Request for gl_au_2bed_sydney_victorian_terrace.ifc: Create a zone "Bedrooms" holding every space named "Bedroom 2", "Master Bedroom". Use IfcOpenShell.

First a look at what the model holds.

```python
import ifcopenshell

model = ifcopenshell.open("gl_au_2bed_sydney_victorian_terrace.ifc")
print(model.schema)
seen = {}
for space in model.by_type("IfcSpace"):
    seen[space.LongName] = seen.get(space.LongName, 0) + 1
for name, count in sorted(seen.items(), key=str):
    print(count, "x", name)
print("zones:", [z.Name for z in model.by_type("IfcZone")][:20])
```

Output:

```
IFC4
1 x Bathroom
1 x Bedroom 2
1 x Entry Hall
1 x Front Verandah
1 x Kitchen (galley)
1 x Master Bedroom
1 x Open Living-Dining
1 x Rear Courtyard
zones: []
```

```python
import ifcopenshell
import ifcopenshell.api.group
import ifcopenshell.api.root

model = ifcopenshell.open("gl_au_2bed_sydney_victorian_terrace.ifc")

names = {"Bedroom 2", "Master Bedroom"}
spaces = [s for s in model.by_type("IfcSpace") if s.LongName in names]

zone = ifcopenshell.api.root.create_entity(model, ifc_class="IfcZone", name="Bedrooms")
ifcopenshell.api.group.assign_group(model, products=spaces, group=zone)
print(len(spaces), "spaces in", zone.Name)

model.write("gl_au_2bed_sydney_victorian_terrace_updated.ifc")
```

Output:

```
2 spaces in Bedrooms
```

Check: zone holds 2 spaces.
